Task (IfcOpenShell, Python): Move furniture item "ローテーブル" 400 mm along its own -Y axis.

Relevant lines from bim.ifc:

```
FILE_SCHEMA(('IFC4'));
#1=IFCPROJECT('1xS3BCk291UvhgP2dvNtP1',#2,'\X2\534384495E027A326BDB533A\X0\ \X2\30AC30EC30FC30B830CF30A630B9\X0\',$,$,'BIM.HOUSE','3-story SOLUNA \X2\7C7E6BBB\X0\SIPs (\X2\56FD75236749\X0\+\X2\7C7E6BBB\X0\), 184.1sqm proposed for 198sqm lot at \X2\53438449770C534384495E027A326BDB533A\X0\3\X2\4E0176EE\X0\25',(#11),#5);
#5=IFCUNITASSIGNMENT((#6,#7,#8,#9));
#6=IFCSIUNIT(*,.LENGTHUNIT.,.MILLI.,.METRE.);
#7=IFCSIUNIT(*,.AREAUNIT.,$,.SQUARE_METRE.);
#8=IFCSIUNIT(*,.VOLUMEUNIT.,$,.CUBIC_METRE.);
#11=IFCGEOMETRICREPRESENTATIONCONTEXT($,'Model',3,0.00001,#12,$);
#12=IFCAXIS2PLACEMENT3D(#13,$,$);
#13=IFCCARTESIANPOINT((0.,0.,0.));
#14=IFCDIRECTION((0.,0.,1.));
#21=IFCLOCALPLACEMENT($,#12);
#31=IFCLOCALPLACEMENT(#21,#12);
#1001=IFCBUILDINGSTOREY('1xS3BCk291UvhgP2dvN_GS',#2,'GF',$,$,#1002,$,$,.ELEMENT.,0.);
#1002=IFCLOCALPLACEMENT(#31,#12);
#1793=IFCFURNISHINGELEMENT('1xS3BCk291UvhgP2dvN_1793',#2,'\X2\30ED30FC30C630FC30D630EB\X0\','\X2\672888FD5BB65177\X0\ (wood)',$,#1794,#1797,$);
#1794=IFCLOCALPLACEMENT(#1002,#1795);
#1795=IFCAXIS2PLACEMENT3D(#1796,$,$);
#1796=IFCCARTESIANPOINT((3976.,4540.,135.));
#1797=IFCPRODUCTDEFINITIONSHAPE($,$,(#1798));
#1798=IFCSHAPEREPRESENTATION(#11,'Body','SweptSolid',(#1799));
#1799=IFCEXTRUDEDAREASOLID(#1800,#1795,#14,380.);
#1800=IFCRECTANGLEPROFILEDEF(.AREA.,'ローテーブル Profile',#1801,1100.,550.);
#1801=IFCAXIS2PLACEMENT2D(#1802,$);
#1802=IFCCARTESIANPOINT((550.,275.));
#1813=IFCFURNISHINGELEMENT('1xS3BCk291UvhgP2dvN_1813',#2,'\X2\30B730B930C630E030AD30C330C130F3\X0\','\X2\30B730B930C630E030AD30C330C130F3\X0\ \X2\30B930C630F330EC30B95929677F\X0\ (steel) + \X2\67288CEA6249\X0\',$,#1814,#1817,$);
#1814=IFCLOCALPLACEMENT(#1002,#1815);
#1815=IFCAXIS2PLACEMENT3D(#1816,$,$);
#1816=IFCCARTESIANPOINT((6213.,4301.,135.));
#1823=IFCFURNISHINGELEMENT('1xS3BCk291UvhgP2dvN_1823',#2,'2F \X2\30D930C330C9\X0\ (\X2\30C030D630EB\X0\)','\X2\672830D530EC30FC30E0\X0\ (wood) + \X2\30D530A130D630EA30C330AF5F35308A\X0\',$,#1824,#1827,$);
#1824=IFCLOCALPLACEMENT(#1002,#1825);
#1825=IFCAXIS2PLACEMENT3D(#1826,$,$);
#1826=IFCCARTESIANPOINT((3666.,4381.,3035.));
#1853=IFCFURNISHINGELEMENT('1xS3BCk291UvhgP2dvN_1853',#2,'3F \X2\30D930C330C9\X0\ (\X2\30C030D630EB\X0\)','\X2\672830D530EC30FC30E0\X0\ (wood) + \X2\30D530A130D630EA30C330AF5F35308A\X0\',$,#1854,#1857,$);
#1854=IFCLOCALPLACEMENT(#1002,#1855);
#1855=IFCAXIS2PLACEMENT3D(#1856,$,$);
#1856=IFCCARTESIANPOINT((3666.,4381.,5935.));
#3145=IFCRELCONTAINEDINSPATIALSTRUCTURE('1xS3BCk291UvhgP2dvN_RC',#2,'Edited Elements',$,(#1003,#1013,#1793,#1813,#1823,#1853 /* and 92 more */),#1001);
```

```python
import ifcopenshell
import ifcopenshell.api.geometry
import ifcopenshell.util.placement

model = ifcopenshell.open("bim.ifc")

item = model.by_guid("1xS3BCk291UvhgP2dvN_1793")
matrix = ifcopenshell.util.placement.get_local_placement(item.ObjectPlacement)
matrix[:3, 3] -= matrix[:3, 1] * 400.0
ifcopenshell.api.geometry.edit_object_placement(model, product=item, matrix=matrix, is_si=False)

print(ifcopenshell.util.placement.get_local_placement(item.ObjectPlacement).round(3) + 0.0)

model.write("bim_updated.ifc")
```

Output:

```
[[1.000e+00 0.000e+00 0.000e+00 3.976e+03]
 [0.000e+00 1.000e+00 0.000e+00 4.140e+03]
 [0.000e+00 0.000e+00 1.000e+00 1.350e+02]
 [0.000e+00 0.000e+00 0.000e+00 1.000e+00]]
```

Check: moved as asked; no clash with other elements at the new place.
